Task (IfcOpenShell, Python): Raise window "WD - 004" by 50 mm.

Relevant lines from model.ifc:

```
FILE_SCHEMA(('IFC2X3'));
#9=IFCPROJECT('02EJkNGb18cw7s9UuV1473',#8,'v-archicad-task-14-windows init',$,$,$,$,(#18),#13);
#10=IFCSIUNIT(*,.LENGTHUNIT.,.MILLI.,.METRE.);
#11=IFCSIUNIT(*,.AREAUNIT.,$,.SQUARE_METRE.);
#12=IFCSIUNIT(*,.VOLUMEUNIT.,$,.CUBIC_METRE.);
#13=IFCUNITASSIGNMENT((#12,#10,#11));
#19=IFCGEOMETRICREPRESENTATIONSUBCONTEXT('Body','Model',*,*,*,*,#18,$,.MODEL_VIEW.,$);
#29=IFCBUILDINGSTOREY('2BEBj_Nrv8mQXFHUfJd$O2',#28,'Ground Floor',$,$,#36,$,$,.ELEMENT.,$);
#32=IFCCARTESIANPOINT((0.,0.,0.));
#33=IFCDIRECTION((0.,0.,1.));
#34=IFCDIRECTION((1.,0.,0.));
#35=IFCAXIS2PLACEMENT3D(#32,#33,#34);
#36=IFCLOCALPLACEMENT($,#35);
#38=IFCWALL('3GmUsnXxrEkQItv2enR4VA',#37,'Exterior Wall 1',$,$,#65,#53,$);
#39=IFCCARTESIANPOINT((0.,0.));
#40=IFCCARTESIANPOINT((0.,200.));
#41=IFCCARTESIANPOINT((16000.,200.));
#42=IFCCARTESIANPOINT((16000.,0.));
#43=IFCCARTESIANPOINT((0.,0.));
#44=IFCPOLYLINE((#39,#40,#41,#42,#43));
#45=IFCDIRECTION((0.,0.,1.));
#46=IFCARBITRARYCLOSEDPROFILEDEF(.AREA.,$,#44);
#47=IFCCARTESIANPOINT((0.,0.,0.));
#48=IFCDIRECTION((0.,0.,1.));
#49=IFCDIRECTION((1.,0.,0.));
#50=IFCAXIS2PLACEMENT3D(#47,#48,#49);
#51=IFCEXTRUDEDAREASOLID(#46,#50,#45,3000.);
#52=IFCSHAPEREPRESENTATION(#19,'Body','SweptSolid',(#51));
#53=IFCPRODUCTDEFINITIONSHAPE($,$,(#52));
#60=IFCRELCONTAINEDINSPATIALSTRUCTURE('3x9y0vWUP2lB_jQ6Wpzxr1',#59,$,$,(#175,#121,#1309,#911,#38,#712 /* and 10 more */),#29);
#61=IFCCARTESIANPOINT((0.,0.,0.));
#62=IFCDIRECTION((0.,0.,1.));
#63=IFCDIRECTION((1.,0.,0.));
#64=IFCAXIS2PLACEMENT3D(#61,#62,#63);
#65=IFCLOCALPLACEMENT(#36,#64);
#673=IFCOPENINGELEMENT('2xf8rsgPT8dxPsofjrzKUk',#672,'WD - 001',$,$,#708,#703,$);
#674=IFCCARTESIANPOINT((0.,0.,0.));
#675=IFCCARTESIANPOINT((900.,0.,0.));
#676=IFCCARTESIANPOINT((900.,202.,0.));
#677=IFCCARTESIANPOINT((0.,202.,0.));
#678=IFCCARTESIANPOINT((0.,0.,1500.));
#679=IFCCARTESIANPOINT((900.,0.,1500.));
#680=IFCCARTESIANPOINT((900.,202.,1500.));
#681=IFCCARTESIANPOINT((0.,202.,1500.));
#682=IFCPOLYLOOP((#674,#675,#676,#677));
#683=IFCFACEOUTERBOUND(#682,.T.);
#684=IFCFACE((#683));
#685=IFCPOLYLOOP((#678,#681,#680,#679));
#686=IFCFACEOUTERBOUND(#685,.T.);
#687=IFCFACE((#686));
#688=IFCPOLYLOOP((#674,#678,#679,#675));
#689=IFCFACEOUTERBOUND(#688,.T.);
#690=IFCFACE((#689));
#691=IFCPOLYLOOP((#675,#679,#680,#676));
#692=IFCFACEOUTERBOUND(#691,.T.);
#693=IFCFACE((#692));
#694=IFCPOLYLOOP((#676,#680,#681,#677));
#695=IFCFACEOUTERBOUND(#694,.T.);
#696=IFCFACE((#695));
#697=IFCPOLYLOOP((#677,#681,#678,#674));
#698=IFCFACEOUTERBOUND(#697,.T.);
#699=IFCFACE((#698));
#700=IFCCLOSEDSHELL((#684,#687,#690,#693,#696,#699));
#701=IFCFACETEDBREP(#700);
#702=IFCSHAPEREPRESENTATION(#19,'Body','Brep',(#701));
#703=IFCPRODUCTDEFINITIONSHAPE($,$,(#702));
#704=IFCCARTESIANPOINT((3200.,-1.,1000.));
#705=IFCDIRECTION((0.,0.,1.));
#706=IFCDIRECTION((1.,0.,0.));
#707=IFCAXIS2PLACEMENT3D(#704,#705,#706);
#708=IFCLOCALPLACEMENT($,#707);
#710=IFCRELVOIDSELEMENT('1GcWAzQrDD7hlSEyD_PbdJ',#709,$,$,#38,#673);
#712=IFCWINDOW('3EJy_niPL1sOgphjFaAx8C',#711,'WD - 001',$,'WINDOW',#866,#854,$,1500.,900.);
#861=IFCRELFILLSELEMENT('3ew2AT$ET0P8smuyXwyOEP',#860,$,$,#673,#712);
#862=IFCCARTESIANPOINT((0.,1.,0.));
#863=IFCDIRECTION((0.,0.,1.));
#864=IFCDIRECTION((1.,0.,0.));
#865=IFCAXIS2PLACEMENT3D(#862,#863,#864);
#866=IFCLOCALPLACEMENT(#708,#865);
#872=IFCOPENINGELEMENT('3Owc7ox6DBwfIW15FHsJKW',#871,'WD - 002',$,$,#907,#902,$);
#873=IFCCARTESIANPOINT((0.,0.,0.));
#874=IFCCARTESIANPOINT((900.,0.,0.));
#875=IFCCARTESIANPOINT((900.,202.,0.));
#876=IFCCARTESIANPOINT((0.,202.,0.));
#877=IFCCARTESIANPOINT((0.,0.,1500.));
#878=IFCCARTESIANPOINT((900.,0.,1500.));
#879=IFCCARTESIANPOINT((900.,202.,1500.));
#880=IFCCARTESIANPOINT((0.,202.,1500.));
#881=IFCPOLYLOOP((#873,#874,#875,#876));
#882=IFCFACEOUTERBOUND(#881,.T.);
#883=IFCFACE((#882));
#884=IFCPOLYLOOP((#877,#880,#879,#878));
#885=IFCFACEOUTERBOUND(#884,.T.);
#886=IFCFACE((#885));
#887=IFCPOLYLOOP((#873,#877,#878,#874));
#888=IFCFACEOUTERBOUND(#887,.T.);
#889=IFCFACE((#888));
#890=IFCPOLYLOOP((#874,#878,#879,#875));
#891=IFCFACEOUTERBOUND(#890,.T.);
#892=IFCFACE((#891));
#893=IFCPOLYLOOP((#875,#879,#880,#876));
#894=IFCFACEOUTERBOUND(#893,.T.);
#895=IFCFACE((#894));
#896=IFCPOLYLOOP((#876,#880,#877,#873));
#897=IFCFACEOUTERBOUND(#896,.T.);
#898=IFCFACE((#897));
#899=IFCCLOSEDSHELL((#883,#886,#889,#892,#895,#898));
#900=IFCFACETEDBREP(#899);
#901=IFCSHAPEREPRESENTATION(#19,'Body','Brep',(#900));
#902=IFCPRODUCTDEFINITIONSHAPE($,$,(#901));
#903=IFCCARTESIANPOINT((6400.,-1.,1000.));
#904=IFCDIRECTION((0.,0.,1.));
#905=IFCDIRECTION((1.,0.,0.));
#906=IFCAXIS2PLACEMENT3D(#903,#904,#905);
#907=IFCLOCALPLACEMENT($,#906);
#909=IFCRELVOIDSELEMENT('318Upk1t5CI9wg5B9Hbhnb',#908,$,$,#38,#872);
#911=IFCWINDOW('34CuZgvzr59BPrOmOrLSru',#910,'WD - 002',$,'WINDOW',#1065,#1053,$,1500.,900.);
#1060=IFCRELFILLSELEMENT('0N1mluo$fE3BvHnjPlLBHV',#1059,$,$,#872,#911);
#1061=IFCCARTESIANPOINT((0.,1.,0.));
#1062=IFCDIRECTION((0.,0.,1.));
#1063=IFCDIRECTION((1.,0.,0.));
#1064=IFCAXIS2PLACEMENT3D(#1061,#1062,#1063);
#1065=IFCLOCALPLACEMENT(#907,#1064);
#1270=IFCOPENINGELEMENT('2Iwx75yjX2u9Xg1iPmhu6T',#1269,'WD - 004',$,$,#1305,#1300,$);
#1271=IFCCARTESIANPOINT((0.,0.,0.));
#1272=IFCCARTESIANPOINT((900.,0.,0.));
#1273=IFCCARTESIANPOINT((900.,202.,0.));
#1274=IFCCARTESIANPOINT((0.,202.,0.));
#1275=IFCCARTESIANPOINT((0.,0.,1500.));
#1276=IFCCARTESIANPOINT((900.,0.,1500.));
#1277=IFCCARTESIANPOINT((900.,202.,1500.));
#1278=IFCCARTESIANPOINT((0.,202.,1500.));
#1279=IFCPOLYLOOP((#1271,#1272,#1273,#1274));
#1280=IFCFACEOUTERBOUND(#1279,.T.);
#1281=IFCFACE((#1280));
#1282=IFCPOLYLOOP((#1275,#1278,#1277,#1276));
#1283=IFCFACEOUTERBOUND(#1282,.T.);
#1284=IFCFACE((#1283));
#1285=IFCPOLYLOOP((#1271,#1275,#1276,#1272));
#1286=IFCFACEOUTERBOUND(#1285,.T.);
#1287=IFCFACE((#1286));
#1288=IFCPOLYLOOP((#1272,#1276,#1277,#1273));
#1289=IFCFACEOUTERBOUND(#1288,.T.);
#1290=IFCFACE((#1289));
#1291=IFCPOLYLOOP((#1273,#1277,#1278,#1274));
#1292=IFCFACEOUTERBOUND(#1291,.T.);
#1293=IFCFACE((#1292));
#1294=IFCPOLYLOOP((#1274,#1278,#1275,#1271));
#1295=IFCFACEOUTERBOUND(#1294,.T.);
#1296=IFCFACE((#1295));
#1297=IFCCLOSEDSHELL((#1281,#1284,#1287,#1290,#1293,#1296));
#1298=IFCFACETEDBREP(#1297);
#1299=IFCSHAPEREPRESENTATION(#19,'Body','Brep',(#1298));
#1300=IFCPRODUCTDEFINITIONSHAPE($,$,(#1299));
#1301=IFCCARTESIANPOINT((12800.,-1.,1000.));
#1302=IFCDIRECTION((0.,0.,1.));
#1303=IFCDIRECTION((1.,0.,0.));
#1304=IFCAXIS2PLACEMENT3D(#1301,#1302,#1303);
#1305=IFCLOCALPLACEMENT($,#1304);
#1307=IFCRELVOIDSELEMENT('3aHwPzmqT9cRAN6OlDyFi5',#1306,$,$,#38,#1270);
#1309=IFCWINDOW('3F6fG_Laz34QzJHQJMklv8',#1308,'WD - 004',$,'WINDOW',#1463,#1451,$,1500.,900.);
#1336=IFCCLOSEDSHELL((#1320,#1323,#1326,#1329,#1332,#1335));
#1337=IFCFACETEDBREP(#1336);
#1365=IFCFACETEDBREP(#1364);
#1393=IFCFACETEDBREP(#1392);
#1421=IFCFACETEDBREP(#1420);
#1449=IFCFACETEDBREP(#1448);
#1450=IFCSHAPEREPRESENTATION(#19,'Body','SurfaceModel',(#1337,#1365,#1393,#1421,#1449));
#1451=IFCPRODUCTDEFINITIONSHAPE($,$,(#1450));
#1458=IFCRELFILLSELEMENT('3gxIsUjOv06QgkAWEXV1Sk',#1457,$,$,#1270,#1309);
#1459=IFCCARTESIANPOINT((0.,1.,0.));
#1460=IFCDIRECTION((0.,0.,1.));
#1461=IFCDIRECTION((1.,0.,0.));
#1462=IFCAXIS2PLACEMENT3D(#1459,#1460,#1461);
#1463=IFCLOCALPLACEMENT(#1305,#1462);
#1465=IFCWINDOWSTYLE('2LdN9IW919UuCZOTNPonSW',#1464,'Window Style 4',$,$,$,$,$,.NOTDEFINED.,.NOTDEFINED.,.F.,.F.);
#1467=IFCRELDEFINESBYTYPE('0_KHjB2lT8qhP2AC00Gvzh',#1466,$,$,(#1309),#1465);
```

```python
import numpy as np
import ifcopenshell
import ifcopenshell.api.geometry
import ifcopenshell.util.placement
import ifcopenshell.util.unit

model = ifcopenshell.open("model.ifc")
unit_scale = ifcopenshell.util.unit.calculate_unit_scale(model)

window = model.by_guid("3F6fG_Laz34QzJHQJMklv8")
opening = window.FillsVoids[0].RelatingOpeningElement
dz = 50.0

shift = np.array([0.0, 0.0, dz])
# The window is placed relative to its opening, so it follows when the opening moves.
matrix = ifcopenshell.util.placement.get_local_placement(opening.ObjectPlacement)
matrix[:3, 3] += shift
ifcopenshell.api.geometry.edit_object_placement(
    model, product=opening, matrix=matrix, is_si=False, should_transform_children=True
)

print(f"moved by {dz * unit_scale:+.3f} m")

model.write("model_rev.ifc")
```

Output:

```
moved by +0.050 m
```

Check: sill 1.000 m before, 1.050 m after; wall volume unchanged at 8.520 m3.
